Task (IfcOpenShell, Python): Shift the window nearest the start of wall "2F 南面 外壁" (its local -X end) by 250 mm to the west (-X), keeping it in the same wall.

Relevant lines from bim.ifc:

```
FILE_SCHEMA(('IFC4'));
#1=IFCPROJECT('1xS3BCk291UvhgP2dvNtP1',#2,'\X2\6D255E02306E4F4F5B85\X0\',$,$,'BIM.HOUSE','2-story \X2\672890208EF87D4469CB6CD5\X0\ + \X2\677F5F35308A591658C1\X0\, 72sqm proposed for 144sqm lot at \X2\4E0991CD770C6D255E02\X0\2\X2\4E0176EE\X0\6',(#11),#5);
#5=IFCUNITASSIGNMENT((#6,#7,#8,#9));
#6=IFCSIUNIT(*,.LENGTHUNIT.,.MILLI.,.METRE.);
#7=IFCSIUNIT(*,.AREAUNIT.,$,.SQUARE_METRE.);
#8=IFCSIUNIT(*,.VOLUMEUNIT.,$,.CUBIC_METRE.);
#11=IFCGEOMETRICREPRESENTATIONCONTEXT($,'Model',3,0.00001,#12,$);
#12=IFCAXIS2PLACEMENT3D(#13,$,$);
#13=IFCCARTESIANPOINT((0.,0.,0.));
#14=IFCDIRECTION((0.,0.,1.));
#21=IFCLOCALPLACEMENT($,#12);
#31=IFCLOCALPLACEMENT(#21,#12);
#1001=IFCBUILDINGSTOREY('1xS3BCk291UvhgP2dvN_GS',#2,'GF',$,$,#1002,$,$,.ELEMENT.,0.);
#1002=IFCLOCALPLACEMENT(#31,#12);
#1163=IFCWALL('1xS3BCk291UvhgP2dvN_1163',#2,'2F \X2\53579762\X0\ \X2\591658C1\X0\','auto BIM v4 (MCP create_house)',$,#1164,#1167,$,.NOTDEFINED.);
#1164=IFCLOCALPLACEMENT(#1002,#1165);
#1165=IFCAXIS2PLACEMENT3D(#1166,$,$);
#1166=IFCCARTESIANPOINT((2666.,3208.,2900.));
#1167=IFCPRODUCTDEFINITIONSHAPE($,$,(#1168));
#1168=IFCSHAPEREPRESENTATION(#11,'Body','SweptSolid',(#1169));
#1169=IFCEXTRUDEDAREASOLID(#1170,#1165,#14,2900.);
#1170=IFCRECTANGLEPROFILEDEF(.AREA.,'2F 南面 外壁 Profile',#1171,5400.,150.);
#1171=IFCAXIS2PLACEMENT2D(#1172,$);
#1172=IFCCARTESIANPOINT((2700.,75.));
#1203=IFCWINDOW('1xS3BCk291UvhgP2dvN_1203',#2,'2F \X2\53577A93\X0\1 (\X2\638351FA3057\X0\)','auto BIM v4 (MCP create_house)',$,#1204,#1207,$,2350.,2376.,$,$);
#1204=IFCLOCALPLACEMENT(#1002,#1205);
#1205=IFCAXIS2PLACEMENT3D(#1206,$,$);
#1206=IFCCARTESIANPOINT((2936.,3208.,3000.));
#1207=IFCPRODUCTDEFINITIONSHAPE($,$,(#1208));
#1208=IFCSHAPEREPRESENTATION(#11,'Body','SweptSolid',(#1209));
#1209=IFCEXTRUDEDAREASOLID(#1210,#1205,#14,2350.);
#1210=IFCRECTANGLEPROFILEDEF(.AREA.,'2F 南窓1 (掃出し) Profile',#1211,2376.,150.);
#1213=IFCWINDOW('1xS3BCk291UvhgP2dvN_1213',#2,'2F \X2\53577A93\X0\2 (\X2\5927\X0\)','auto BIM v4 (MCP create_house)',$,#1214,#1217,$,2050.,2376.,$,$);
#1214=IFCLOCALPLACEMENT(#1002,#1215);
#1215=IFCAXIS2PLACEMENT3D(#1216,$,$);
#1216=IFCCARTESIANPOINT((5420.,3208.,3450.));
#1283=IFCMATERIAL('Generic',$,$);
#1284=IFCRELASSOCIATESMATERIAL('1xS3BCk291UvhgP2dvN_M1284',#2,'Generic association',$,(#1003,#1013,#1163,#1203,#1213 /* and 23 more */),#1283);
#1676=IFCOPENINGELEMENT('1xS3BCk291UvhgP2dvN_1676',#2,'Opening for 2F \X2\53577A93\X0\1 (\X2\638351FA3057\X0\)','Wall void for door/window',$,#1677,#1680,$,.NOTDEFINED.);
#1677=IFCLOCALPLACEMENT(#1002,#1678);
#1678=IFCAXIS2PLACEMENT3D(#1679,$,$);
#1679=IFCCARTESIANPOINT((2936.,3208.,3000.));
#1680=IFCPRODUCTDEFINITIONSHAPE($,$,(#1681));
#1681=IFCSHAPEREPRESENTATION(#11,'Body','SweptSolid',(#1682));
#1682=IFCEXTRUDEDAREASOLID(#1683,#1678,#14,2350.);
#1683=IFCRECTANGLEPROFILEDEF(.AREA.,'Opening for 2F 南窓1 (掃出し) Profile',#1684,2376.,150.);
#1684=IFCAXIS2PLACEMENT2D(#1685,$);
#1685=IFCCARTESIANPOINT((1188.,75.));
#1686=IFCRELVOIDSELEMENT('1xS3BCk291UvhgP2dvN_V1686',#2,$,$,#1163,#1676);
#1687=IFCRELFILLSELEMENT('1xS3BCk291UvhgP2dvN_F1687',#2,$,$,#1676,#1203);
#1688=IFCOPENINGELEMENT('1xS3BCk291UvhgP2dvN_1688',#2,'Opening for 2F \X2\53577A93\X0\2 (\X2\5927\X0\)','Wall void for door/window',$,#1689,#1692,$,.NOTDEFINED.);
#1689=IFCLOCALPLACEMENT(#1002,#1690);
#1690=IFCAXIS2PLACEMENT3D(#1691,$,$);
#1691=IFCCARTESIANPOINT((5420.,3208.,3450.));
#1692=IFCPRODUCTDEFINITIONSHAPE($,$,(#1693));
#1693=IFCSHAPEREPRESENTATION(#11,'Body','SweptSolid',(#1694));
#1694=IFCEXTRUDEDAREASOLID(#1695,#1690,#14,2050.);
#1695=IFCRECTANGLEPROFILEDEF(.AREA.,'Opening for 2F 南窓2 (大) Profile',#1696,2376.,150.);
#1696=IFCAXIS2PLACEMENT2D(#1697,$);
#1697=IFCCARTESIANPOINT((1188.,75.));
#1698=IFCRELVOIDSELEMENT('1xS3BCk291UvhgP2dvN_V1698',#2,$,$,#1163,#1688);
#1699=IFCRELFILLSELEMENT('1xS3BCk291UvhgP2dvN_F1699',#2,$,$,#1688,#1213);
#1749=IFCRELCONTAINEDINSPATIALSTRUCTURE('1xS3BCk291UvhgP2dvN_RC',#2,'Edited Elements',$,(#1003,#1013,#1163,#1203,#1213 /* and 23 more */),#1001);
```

```python
import ifcopenshell
import ifcopenshell.api.geometry
import ifcopenshell.util.placement

model = ifcopenshell.open("bim.ifc")

window = model.by_guid("1xS3BCk291UvhgP2dvN_1203")
opening = window.FillsVoids[0].RelatingOpeningElement
wall = opening.VoidsElements[0].RelatingBuildingElement

wall_matrix = ifcopenshell.util.placement.get_local_placement(wall.ObjectPlacement)
shift = wall_matrix[:3, 0] * -250.0
before = ifcopenshell.util.placement.get_local_placement(window.ObjectPlacement)[:3, 3].copy()

# The window is not placed relative to its opening, so move both.
for product in (opening, window):
    matrix = ifcopenshell.util.placement.get_local_placement(product.ObjectPlacement)
    matrix[:3, 3] += shift
    ifcopenshell.api.geometry.edit_object_placement(model, product=product, matrix=matrix, is_si=False)

after = ifcopenshell.util.placement.get_local_placement(window.ObjectPlacement)[:3, 3]
print("window moved by", (after - before).round(3) + 0.0)

model.write("bim_updated.ifc")
```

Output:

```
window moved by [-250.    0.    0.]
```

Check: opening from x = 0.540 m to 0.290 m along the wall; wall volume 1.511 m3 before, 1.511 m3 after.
